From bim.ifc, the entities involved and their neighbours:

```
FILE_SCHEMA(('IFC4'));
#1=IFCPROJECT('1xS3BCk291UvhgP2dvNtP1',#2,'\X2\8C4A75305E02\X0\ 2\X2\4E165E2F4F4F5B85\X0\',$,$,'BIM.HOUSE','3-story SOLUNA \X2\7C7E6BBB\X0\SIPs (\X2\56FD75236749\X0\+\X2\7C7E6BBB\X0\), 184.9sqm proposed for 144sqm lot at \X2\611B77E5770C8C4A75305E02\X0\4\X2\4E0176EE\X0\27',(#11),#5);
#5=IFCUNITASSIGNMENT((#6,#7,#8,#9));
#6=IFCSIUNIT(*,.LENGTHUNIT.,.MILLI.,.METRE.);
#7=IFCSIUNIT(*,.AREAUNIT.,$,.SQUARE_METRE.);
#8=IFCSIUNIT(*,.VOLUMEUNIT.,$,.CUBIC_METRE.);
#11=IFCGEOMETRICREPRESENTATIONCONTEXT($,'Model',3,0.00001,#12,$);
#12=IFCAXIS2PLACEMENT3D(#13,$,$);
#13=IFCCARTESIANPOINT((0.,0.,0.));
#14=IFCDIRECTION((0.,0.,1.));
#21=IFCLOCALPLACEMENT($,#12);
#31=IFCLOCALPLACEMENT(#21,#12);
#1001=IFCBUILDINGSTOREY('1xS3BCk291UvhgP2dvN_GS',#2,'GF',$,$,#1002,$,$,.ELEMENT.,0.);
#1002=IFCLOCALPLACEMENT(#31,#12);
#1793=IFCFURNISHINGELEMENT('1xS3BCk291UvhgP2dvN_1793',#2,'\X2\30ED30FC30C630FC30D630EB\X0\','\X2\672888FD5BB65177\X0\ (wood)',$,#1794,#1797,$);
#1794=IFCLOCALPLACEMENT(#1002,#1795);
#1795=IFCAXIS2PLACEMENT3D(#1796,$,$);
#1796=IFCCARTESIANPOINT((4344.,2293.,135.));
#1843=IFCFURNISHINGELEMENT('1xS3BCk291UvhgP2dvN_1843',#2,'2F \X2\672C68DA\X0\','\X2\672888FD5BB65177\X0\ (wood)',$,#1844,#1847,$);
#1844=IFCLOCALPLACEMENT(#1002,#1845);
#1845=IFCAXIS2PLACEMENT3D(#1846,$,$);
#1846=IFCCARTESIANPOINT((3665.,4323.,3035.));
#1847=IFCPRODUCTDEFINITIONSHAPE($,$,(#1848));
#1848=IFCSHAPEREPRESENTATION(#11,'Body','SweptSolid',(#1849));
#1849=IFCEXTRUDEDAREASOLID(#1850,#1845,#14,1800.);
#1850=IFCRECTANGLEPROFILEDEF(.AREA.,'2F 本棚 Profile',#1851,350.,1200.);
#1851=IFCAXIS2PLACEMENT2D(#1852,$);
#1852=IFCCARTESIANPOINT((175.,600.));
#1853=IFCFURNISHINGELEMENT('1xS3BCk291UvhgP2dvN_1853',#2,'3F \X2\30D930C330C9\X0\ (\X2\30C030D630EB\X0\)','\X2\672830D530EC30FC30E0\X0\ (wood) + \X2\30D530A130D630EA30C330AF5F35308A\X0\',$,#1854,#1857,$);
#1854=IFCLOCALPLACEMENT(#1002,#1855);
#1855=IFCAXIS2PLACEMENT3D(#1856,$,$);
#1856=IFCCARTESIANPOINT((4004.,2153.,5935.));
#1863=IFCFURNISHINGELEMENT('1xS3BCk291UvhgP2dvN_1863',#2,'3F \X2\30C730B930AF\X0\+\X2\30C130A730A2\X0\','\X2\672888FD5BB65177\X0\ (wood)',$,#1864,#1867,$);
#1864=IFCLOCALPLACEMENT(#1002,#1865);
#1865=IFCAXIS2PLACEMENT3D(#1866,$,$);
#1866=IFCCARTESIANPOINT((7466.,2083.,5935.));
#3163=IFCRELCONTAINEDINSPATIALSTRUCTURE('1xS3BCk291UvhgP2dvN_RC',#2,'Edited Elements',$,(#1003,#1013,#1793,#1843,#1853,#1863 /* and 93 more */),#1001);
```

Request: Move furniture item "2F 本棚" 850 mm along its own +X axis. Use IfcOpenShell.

```python
import ifcopenshell
import ifcopenshell.api.geometry
import ifcopenshell.util.placement
import ifcopenshell.util.unit

model = ifcopenshell.open("bim.ifc")
unit_scale = ifcopenshell.util.unit.calculate_unit_scale(model)

item = model.by_guid("1xS3BCk291UvhgP2dvN_1843")
matrix = ifcopenshell.util.placement.get_local_placement(item.ObjectPlacement)
matrix[:3, 3] += matrix[:3, 0] * 0.85 / unit_scale
ifcopenshell.api.geometry.edit_object_placement(model, product=item, matrix=matrix, is_si=False)

print(ifcopenshell.util.placement.get_local_placement(item.ObjectPlacement).round(3) + 0.0)

model.write("bim-out.ifc")
```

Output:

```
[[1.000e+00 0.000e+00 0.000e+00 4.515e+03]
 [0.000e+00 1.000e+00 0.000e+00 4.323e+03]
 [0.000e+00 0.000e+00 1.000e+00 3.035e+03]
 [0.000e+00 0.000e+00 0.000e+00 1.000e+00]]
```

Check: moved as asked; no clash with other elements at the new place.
